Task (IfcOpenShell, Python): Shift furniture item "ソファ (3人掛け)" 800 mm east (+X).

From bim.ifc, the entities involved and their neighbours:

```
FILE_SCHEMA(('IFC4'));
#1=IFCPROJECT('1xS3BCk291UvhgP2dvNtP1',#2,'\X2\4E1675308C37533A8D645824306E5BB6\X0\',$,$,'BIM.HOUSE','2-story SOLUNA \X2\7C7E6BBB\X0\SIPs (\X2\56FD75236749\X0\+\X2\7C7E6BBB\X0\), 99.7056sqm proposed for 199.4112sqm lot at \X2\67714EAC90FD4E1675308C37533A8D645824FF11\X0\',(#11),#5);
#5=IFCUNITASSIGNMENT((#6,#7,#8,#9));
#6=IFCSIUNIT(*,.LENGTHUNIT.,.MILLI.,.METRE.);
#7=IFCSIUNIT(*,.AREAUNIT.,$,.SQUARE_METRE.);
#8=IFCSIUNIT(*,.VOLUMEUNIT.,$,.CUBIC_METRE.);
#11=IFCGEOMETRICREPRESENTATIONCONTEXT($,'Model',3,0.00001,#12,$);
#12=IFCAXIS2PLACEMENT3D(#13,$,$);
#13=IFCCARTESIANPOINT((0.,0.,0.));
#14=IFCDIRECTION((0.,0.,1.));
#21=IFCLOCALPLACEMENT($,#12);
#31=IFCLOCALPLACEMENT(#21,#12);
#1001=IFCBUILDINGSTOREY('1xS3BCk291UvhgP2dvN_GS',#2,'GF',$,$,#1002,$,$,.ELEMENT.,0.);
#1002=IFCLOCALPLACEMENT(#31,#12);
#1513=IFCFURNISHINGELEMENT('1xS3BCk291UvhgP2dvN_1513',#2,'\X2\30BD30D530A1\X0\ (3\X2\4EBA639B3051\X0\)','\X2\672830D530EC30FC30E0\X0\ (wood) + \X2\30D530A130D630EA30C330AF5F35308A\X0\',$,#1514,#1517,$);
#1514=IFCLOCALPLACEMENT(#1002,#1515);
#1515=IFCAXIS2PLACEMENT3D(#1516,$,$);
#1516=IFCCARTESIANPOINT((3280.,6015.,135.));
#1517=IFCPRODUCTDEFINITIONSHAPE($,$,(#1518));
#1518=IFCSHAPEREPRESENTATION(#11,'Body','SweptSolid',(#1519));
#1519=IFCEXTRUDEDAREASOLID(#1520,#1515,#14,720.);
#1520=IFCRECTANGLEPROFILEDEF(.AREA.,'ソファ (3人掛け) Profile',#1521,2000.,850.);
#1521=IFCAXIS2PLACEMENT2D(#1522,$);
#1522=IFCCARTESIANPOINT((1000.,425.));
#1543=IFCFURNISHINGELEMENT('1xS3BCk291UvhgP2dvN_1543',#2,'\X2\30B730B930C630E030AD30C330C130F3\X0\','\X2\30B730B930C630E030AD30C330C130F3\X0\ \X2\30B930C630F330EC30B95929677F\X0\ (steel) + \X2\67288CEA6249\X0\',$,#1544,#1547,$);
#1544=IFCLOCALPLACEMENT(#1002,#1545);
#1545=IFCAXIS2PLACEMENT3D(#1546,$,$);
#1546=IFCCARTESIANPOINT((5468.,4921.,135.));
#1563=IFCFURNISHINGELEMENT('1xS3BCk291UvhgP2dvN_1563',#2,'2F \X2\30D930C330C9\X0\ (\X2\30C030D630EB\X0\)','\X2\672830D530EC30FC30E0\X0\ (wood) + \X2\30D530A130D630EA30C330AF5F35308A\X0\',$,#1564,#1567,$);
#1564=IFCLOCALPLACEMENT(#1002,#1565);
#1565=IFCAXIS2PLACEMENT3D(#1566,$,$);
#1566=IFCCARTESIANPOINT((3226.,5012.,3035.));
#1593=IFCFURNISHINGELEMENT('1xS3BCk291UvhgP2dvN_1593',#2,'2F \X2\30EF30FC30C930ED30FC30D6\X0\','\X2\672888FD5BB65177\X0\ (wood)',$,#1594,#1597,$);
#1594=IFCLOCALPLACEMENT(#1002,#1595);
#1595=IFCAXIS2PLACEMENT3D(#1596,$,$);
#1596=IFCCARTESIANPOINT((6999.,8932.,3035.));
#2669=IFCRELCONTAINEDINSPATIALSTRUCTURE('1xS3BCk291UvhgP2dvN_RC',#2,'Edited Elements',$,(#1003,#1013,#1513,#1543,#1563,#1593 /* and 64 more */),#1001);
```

```python
import ifcopenshell
import ifcopenshell.api.geometry
import ifcopenshell.util.placement
import ifcopenshell.util.unit

model = ifcopenshell.open("bim.ifc")
unit_scale = ifcopenshell.util.unit.calculate_unit_scale(model)

item = model.by_id(1513)
matrix = ifcopenshell.util.placement.get_local_placement(item.ObjectPlacement)
matrix[0, 3] += 0.8 / unit_scale
ifcopenshell.api.geometry.edit_object_placement(model, product=item, matrix=matrix, is_si=False)

print(ifcopenshell.util.placement.get_local_placement(item.ObjectPlacement).round(3) + 0.0)

model.write("bim-out.ifc")
```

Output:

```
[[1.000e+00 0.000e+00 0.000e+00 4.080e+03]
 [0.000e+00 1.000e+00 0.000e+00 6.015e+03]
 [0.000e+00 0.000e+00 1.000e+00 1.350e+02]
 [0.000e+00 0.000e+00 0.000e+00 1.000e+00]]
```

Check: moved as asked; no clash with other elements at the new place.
